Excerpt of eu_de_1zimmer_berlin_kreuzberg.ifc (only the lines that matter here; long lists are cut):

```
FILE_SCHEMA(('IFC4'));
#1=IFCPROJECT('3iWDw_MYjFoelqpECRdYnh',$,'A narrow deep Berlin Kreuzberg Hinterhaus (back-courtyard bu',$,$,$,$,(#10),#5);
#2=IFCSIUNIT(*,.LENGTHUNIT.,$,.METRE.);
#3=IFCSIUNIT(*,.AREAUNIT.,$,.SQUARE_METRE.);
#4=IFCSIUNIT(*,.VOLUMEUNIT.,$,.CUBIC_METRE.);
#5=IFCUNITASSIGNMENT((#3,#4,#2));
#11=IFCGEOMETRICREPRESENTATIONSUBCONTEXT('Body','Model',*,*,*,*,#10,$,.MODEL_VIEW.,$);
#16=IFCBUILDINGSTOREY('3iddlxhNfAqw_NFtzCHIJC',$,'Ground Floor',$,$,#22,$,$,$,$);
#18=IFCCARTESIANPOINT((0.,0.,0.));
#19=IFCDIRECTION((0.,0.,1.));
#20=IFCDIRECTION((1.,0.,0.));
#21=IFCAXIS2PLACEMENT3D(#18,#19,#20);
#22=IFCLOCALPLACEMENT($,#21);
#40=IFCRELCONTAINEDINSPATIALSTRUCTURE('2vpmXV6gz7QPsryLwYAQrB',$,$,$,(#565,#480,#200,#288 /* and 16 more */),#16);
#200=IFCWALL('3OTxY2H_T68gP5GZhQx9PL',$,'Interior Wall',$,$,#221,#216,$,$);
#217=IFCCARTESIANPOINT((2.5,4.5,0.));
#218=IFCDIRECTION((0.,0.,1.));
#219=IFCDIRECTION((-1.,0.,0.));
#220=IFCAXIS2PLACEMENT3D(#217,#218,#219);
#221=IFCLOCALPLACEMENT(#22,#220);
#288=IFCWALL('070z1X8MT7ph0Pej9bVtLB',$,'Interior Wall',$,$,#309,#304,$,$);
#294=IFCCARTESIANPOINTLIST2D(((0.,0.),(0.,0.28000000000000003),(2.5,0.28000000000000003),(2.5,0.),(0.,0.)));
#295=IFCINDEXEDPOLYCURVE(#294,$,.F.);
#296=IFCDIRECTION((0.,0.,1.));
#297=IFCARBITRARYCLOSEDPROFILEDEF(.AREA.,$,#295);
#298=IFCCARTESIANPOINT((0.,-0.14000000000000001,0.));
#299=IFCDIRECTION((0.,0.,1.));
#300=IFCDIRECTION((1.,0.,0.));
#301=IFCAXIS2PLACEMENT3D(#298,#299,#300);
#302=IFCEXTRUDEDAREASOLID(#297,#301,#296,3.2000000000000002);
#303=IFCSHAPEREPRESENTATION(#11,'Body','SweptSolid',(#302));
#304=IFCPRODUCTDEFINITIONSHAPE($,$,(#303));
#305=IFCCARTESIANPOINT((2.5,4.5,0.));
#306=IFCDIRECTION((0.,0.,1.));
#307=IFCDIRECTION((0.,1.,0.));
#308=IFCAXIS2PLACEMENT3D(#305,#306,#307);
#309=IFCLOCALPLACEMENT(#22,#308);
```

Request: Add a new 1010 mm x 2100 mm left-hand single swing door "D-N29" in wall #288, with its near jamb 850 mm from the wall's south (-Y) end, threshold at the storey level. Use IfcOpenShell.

```python
import numpy as np
import ifcopenshell
import ifcopenshell.api.feature
import ifcopenshell.api.geometry
import ifcopenshell.api.root
import ifcopenshell.api.spatial
import ifcopenshell.geom
import ifcopenshell.util.element
import ifcopenshell.util.placement
import ifcopenshell.util.representation
import ifcopenshell.util.shape
import ifcopenshell.util.unit

model = ifcopenshell.open("eu_de_1zimmer_berlin_kreuzberg.ifc")
unit_scale = ifcopenshell.util.unit.calculate_unit_scale(model)
settings = ifcopenshell.geom.settings()


def volume(element):
    """Net volume in cubic metres, openings subtracted."""
    shape = ifcopenshell.geom.create_shape(settings, element)
    return ifcopenshell.util.shape.get_volume(shape.geometry)


wall = model.by_id(288)
storey = ifcopenshell.util.element.get_container(wall, ifc_class="IfcBuildingStorey")
context = ifcopenshell.util.representation.get_context(model, "Model", "Body", "MODEL_VIEW")
before = volume(wall)

width, height, from_end, sill = 1.01, 2.1, 0.85, 0.0  # metres

# The wall runs along its own X axis, and the end named is its -X end.
wall_shape = ifcopenshell.geom.create_shape(settings, wall)
x, y, z = ifcopenshell.util.shape.get_vertices(wall_shape.geometry).T
start = x.min() + from_end
face, thickness = float(y.min()), float(y.max() - y.min())
wall_matrix = ifcopenshell.util.placement.get_local_placement(wall.ObjectPlacement)
level = ifcopenshell.util.placement.get_local_placement(storey.ObjectPlacement)[2, 3]


def in_wall(x, y):
    """Placement at x, y metres in the wall's axes, at sill height."""
    matrix = wall_matrix.copy()
    matrix[:, 3] = wall_matrix @ np.array([x / unit_scale, y / unit_scale, 0.0, 1.0])
    matrix[2, 3] = level + sill / unit_scale
    return matrix


# Opening: a box that overshoots both wall faces by 50 mm.
opening = ifcopenshell.api.root.create_entity(model, ifc_class="IfcOpeningElement", predefined_type="OPENING")
box = ifcopenshell.api.geometry.add_wall_representation(
    model, context=context, length=width, height=height, thickness=thickness + 0.1
)
ifcopenshell.api.geometry.assign_representation(model, product=opening, representation=box)
ifcopenshell.api.geometry.edit_object_placement(model, product=opening, matrix=in_wall(start, face - 0.05), is_si=False)
ifcopenshell.api.feature.add_feature(model, feature=opening, element=wall)

door = ifcopenshell.api.root.create_entity(model, ifc_class="IfcDoor", name="D-N29", predefined_type="DOOR")
door.OverallWidth, door.OverallHeight = width / unit_scale, height / unit_scale
door.OperationType = "SINGLE_SWING_LEFT"
body = ifcopenshell.api.geometry.add_door_representation(
    model,
    context=context,
    overall_width=door.OverallWidth,
    overall_height=door.OverallHeight,
    operation_type="SINGLE_SWING_LEFT",
    lining_properties={"LiningDepth": thickness / unit_scale, "ThresholdDepth": thickness / unit_scale},
)
ifcopenshell.api.geometry.assign_representation(model, product=door, representation=body)
ifcopenshell.api.spatial.assign_container(model, products=[door], relating_structure=storey)
ifcopenshell.api.feature.add_filling(model, opening=opening, element=door)

# The lining spans the wall, so the door starts at the wall face.
ifcopenshell.api.geometry.edit_object_placement(model, product=door, matrix=in_wall(start, face), is_si=False)

after = volume(wall)

print(f"wall volume {before:.3f} -> {after:.3f} m3")

model.write("eu_de_1zimmer_berlin_kreuzberg_updated.ifc")
```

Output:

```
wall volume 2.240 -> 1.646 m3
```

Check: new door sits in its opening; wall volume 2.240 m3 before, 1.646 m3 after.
